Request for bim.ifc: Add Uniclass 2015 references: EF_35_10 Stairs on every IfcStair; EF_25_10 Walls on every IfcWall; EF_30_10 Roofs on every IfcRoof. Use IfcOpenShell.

First a look at what the model holds.

```python
import ifcopenshell

model = ifcopenshell.open("bim.ifc")
print(model.schema)
print("classifications:", [c.Name for c in model.by_type("IfcClassification")])
for ifc_class in ("IfcDoor", "IfcRoof", "IfcStair", "IfcWall", "IfcWindow"):
    print(ifc_class, len(model.by_type(ifc_class)))
```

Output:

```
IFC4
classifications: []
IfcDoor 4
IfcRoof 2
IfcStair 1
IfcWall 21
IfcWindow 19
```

```python
import ifcopenshell
import ifcopenshell.api.classification

model = ifcopenshell.open("bim.ifc")

system = ifcopenshell.api.classification.add_classification(model, classification="Uniclass 2015")

codes = {
    "IfcStair": ("EF_35_10", "Stairs"),
    "IfcWall": ("EF_25_10", "Walls"),
    "IfcRoof": ("EF_30_10", "Roofs"),
}
for ifc_class, (code, name) in codes.items():
    products = model.by_type(ifc_class)
    ifcopenshell.api.classification.add_reference(
        model, products=products, classification=system, identification=code, name=name
    )
    print(code, len(products))

model.write("bim-out.ifc")
```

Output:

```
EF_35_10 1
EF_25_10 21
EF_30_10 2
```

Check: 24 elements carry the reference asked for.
